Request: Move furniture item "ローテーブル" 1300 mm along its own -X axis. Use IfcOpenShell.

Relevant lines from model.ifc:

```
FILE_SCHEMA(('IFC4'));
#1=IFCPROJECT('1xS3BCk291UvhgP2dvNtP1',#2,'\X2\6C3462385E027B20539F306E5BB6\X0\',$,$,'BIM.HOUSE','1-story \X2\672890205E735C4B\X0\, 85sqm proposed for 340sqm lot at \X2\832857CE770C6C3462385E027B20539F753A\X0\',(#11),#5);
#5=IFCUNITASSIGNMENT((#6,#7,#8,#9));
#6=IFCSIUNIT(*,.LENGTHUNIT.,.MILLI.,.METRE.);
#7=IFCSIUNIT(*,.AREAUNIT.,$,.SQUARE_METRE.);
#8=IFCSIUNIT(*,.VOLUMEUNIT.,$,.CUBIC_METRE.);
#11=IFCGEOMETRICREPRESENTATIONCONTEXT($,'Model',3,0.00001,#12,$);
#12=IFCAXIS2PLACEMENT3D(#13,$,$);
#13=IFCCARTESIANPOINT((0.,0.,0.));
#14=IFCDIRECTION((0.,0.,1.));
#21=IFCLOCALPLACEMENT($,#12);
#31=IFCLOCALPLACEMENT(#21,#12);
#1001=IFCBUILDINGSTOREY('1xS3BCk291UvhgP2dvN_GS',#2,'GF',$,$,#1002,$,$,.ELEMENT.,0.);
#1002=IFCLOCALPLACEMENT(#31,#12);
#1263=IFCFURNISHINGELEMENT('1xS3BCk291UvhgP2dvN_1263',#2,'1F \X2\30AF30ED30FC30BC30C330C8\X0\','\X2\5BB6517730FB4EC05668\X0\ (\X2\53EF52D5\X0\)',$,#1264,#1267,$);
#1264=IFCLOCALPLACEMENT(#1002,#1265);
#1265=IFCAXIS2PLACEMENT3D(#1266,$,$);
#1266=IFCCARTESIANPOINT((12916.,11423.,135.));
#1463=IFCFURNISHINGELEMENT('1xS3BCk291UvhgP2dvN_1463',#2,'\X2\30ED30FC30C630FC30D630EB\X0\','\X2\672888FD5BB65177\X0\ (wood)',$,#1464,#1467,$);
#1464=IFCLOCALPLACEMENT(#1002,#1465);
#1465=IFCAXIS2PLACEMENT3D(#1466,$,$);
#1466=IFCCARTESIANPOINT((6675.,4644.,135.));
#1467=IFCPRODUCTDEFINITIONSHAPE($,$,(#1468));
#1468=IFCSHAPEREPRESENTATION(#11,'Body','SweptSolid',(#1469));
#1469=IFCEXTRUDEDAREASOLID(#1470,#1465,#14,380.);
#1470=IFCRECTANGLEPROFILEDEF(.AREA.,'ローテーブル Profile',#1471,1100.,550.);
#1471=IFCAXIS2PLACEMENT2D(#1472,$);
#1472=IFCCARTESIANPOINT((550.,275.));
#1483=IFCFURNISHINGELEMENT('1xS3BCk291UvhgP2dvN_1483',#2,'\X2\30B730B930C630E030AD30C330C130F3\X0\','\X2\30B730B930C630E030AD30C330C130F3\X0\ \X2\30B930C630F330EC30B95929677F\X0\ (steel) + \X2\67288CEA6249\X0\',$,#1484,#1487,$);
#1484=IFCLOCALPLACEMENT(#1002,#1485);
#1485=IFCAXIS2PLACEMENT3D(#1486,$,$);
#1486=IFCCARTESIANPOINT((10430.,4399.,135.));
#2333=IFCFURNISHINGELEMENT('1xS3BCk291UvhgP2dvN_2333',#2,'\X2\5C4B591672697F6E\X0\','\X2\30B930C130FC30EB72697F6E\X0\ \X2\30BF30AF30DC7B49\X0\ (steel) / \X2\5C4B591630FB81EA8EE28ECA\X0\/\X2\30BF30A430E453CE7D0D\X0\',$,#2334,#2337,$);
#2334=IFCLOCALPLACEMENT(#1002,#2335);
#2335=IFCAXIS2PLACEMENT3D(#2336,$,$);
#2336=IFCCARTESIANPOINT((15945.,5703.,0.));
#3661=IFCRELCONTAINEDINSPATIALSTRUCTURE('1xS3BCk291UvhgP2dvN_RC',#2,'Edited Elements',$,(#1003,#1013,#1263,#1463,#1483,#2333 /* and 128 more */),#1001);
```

```python
import ifcopenshell
import ifcopenshell.api.geometry
import ifcopenshell.util.placement
import ifcopenshell.util.unit

model = ifcopenshell.open("model.ifc")
unit_scale = ifcopenshell.util.unit.calculate_unit_scale(model)

item = model.by_id(1463)
matrix = ifcopenshell.util.placement.get_local_placement(item.ObjectPlacement)
matrix[:3, 3] -= matrix[:3, 0] * 1.3 / unit_scale
ifcopenshell.api.geometry.edit_object_placement(model, product=item, matrix=matrix, is_si=False)

print(ifcopenshell.util.placement.get_local_placement(item.ObjectPlacement).round(3) + 0.0)

model.write("model_v2.ifc")
```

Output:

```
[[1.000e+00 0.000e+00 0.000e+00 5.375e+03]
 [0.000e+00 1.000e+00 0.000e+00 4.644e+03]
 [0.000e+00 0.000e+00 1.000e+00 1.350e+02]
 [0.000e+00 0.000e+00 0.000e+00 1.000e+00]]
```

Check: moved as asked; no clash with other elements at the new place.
